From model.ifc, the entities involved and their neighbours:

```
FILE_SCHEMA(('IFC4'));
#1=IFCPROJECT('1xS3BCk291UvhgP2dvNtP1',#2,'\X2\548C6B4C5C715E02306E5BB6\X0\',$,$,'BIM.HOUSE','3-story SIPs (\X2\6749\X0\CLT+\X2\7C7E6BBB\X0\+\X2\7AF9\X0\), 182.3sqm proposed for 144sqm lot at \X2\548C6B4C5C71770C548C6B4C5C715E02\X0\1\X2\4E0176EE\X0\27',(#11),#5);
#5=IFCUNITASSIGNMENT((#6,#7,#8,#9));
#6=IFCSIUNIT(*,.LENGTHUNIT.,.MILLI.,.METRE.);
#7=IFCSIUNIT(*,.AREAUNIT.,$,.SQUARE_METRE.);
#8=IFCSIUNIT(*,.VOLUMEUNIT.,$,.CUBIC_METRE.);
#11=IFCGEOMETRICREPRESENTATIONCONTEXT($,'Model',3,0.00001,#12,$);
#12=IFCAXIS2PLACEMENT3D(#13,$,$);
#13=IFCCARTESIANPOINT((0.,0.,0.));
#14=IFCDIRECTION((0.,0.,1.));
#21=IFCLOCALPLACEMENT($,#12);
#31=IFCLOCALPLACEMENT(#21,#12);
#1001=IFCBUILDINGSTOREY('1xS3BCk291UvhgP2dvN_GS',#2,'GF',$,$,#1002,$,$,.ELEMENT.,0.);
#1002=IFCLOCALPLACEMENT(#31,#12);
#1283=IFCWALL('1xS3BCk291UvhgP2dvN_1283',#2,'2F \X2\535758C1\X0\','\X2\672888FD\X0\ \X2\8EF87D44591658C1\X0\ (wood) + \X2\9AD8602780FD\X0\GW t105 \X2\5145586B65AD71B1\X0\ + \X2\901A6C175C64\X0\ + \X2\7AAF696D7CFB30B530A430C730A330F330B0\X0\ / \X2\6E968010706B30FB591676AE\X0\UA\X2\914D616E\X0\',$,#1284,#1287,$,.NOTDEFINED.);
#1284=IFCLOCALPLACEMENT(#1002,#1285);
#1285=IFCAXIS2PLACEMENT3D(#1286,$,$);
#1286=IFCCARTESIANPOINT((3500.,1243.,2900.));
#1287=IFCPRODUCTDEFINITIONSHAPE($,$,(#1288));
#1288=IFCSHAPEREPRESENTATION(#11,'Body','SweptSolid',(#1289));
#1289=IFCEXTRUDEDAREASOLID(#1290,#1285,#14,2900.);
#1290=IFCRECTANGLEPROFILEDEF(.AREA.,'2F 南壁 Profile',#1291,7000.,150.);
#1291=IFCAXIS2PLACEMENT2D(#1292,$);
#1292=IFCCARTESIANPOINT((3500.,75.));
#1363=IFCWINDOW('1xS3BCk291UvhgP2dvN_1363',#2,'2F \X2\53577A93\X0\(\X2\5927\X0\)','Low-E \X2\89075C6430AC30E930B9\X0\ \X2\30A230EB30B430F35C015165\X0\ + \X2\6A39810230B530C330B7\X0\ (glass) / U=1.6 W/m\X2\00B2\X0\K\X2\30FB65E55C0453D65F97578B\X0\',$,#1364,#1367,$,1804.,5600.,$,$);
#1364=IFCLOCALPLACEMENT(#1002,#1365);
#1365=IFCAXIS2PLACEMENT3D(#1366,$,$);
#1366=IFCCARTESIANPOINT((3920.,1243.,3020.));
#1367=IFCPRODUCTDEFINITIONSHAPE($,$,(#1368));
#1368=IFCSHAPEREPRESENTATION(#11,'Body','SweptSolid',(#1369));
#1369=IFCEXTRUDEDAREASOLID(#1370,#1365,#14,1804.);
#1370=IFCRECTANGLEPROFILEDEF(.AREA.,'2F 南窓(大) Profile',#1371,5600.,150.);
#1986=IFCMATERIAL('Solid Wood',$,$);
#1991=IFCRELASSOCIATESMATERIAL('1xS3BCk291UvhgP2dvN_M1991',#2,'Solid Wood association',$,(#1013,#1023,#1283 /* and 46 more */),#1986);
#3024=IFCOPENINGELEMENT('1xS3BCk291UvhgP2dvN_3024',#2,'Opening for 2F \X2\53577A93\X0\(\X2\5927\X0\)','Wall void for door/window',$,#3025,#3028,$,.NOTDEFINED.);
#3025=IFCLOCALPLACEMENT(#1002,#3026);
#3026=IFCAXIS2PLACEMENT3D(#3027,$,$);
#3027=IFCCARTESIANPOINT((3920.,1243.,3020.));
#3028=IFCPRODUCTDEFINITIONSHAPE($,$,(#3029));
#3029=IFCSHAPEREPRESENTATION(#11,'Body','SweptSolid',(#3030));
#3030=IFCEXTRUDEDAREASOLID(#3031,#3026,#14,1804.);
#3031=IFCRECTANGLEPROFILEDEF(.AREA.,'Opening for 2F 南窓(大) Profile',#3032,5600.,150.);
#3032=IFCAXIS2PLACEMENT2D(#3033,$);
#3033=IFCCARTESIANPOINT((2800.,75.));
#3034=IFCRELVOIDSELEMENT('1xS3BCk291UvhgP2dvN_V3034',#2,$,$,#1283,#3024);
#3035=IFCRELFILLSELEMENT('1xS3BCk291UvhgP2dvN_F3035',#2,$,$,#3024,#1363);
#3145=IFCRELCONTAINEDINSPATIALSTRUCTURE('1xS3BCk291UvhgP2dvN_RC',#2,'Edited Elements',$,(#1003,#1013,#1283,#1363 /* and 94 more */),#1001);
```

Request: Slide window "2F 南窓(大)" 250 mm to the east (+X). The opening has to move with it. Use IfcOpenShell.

```python
import ifcopenshell
import ifcopenshell.api.geometry
import ifcopenshell.util.placement
import ifcopenshell.util.unit

model = ifcopenshell.open("model.ifc")
unit_scale = ifcopenshell.util.unit.calculate_unit_scale(model)

window = model.by_id(1363)
opening = window.FillsVoids[0].RelatingOpeningElement
wall = opening.VoidsElements[0].RelatingBuildingElement

wall_matrix = ifcopenshell.util.placement.get_local_placement(wall.ObjectPlacement)
shift = wall_matrix[:3, 0] * 0.25 / unit_scale
before = ifcopenshell.util.placement.get_local_placement(window.ObjectPlacement)[:3, 3].copy()

# The window is not placed relative to its opening, so move both.
for product in (opening, window):
    matrix = ifcopenshell.util.placement.get_local_placement(product.ObjectPlacement)
    matrix[:3, 3] += shift
    ifcopenshell.api.geometry.edit_object_placement(model, product=product, matrix=matrix, is_si=False)

after = ifcopenshell.util.placement.get_local_placement(window.ObjectPlacement)[:3, 3]
print("window moved by", (after - before).round(3) + 0.0)

model.write("model_edited.ifc")
```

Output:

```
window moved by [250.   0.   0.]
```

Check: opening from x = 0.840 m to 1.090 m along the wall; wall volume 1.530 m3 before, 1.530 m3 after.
